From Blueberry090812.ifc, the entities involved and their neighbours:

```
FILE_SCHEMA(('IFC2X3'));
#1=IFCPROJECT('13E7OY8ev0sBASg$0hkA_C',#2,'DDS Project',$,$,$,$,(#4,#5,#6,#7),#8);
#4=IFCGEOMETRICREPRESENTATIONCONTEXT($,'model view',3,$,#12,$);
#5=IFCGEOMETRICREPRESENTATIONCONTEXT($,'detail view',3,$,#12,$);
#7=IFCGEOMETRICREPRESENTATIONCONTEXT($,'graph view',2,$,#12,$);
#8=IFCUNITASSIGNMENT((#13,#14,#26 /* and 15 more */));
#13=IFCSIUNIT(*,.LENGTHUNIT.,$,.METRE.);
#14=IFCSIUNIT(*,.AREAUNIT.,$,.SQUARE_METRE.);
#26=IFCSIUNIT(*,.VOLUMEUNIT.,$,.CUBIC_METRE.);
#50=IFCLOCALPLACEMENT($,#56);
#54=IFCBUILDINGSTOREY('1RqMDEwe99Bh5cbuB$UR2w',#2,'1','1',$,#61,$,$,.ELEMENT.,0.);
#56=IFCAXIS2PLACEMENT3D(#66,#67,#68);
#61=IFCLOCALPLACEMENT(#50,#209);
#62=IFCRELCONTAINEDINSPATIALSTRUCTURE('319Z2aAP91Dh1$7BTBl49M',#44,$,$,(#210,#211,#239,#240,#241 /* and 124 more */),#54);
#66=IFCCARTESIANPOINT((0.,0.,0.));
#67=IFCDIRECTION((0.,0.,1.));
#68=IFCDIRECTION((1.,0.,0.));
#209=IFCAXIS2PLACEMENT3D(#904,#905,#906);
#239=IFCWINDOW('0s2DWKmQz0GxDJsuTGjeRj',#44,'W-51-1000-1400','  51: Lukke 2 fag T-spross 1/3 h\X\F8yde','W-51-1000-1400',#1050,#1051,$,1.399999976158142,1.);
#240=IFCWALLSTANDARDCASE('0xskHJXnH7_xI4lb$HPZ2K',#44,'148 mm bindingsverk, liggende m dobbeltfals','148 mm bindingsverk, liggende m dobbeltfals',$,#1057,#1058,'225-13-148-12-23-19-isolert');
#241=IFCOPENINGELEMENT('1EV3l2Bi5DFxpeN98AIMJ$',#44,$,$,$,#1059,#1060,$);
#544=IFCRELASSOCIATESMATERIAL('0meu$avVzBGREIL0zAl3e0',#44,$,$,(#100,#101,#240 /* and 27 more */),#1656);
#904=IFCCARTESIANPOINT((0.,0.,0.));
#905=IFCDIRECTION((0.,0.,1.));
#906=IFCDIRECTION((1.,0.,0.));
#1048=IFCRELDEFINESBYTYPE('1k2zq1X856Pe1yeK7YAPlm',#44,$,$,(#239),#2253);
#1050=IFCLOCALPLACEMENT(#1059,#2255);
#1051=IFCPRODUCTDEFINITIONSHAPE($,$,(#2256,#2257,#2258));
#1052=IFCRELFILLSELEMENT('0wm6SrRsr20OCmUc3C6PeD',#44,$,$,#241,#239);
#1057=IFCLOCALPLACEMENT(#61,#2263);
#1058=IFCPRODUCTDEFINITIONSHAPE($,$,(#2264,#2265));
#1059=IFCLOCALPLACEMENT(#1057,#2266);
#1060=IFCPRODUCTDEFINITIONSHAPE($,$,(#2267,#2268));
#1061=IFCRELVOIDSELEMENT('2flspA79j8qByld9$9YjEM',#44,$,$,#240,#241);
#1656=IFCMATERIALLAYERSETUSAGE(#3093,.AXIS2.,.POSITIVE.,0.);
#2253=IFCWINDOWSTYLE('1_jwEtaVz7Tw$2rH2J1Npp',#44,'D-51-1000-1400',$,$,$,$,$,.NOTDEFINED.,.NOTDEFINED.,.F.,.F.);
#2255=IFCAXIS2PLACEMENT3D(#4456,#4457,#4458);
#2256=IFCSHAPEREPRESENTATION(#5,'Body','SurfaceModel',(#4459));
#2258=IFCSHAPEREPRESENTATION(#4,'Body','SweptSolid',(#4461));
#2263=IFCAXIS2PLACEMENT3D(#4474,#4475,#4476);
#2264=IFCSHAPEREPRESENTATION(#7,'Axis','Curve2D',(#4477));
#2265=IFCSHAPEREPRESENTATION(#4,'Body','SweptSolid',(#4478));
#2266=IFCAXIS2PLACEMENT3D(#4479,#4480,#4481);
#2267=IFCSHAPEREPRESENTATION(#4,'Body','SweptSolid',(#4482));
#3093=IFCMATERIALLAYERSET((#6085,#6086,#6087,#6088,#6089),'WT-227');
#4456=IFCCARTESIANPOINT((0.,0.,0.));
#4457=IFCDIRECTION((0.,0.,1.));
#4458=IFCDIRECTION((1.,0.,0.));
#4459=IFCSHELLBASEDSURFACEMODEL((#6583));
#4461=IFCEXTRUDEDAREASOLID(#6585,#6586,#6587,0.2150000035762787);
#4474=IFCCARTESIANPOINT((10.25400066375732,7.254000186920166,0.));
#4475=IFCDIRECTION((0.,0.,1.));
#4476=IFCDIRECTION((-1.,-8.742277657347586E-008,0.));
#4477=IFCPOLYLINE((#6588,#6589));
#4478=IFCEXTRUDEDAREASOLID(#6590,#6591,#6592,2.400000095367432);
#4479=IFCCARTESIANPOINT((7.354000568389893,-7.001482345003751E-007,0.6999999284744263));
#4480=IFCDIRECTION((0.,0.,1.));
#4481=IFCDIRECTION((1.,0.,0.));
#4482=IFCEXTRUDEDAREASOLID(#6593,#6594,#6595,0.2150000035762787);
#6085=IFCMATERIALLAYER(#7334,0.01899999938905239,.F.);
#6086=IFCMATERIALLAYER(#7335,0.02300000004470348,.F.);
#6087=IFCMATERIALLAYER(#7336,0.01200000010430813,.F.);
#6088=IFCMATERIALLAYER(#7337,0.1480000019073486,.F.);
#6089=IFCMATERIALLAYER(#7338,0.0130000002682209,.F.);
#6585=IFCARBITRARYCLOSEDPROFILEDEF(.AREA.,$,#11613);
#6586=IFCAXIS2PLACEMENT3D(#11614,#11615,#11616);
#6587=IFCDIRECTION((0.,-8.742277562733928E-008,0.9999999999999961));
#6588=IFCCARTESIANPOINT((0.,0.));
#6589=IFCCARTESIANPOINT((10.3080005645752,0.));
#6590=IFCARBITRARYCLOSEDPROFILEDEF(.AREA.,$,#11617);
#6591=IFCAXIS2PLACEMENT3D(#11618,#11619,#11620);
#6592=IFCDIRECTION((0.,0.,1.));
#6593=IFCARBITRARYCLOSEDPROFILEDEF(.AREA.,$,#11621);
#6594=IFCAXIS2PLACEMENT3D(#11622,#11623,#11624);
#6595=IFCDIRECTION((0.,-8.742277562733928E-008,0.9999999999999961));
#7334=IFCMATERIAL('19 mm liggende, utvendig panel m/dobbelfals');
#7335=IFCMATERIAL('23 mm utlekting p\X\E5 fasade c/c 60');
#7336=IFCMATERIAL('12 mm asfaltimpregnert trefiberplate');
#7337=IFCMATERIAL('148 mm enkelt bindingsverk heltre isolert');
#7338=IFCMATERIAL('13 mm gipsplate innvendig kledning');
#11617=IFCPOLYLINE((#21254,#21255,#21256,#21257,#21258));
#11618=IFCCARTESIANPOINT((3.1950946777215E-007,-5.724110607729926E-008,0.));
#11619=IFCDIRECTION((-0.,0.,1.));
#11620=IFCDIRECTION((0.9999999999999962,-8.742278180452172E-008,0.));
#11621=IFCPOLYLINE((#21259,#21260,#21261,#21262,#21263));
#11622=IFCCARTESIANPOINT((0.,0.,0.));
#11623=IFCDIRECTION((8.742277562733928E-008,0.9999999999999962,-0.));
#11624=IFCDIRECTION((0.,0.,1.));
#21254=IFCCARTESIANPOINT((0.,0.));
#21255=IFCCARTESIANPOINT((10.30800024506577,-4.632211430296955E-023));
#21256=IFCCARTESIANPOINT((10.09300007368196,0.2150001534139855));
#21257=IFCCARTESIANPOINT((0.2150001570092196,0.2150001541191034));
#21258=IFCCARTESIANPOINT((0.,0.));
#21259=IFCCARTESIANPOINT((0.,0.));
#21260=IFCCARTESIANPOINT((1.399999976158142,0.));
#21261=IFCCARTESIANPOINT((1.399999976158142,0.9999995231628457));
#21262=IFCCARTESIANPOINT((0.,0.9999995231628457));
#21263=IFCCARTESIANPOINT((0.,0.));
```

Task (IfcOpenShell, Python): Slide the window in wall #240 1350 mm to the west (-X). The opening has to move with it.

```python
import ifcopenshell
import ifcopenshell.api.geometry
import ifcopenshell.util.placement
import ifcopenshell.util.unit

model = ifcopenshell.open("Blueberry090812.ifc")
unit_scale = ifcopenshell.util.unit.calculate_unit_scale(model)

window = model.by_guid("0s2DWKmQz0GxDJsuTGjeRj")
opening = window.FillsVoids[0].RelatingOpeningElement
wall = opening.VoidsElements[0].RelatingBuildingElement

wall_matrix = ifcopenshell.util.placement.get_local_placement(wall.ObjectPlacement)
shift = wall_matrix[:3, 0] * 1.35 / unit_scale
before = ifcopenshell.util.placement.get_local_placement(window.ObjectPlacement)[:3, 3].copy()

# The window is placed relative to its opening, so it follows when the opening moves.
matrix = ifcopenshell.util.placement.get_local_placement(opening.ObjectPlacement)
matrix[:3, 3] += shift
ifcopenshell.api.geometry.edit_object_placement(
    model, product=opening, matrix=matrix, is_si=False, should_transform_children=True
)

after = ifcopenshell.util.placement.get_local_placement(window.ObjectPlacement)[:3, 3]
print("window moved by", (after - before).round(3) + 0.0)

model.write("Blueberry090812_v2.ifc")
```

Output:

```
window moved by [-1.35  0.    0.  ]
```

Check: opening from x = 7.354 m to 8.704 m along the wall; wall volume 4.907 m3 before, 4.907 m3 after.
